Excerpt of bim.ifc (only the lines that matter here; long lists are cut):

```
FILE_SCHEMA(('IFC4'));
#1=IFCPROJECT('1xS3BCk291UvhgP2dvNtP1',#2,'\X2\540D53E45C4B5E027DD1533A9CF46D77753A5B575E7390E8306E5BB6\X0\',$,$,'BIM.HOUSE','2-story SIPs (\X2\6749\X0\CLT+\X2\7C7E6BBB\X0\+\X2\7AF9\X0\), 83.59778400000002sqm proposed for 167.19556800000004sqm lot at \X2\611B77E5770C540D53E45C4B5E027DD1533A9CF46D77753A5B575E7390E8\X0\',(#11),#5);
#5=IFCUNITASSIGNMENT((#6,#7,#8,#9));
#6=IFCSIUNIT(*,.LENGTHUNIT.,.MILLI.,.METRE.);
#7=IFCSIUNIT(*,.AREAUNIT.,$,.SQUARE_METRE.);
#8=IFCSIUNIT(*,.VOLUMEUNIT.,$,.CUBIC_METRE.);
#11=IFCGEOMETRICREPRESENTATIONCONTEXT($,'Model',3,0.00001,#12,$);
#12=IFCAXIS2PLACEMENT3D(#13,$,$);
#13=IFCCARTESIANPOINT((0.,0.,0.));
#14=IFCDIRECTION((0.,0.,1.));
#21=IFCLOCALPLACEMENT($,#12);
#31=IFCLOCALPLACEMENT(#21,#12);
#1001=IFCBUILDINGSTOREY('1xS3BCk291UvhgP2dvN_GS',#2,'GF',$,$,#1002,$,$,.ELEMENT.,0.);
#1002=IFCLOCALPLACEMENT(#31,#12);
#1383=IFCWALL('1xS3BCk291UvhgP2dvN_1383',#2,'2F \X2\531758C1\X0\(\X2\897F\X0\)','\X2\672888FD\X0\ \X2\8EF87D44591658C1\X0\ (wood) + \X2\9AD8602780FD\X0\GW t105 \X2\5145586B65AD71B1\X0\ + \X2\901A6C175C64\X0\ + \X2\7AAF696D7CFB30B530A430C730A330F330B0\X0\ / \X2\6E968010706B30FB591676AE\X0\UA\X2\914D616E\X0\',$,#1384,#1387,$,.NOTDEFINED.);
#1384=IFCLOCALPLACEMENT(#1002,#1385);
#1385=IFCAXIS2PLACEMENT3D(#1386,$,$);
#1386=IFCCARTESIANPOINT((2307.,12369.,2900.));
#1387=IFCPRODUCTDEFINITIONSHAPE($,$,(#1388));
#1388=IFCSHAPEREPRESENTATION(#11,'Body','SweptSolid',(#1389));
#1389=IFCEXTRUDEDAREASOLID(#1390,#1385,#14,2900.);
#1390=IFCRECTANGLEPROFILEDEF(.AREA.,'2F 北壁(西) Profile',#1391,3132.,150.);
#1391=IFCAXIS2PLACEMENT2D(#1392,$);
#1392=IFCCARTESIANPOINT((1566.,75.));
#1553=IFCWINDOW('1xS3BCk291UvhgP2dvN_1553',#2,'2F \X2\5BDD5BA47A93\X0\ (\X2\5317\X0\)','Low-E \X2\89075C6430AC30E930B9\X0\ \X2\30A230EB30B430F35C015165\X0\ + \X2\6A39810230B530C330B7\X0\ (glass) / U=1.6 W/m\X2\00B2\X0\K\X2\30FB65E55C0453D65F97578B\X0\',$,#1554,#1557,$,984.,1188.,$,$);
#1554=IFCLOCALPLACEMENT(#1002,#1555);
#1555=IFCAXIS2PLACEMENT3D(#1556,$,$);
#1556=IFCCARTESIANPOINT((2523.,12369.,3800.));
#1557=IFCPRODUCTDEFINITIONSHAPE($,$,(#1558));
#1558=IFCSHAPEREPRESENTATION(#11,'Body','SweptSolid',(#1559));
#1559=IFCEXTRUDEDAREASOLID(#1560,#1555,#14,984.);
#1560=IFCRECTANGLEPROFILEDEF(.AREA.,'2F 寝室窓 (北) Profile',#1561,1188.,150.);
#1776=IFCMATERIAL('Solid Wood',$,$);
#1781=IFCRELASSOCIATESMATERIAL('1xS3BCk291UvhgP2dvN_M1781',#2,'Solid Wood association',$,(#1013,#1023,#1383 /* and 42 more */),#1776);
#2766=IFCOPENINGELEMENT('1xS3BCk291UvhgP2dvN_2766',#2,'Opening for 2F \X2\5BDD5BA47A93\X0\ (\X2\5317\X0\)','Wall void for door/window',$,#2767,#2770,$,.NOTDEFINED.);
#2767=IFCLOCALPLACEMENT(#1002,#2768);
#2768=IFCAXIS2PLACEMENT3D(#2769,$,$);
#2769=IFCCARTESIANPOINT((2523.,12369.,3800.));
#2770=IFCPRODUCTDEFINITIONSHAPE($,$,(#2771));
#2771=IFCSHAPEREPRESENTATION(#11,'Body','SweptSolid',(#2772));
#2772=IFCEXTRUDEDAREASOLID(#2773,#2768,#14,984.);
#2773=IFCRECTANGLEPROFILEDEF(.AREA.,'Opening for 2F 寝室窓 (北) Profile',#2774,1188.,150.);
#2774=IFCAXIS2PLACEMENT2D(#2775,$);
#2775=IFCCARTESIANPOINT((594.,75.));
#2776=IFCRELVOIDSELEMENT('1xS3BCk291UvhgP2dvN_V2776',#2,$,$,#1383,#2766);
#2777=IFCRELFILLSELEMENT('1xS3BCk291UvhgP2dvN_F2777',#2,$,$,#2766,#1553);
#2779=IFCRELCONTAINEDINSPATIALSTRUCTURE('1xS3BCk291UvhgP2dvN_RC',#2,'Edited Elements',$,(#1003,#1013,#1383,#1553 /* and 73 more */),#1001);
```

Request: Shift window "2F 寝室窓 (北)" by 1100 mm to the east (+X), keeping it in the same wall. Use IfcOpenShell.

```python
import ifcopenshell
import ifcopenshell.api.geometry
import ifcopenshell.util.placement

model = ifcopenshell.open("bim.ifc")

window = model.by_id(1553)
opening = window.FillsVoids[0].RelatingOpeningElement
wall = opening.VoidsElements[0].RelatingBuildingElement

wall_matrix = ifcopenshell.util.placement.get_local_placement(wall.ObjectPlacement)
shift = wall_matrix[:3, 0] * 1100.0
before = ifcopenshell.util.placement.get_local_placement(window.ObjectPlacement)[:3, 3].copy()

# The window is not placed relative to its opening, so move both.
for product in (opening, window):
    matrix = ifcopenshell.util.placement.get_local_placement(product.ObjectPlacement)
    matrix[:3, 3] += shift
    ifcopenshell.api.geometry.edit_object_placement(model, product=product, matrix=matrix, is_si=False)

after = ifcopenshell.util.placement.get_local_placement(window.ObjectPlacement)[:3, 3]
print("window moved by", (after - before).round(3) + 0.0)

model.write("bim_v2.ifc")
```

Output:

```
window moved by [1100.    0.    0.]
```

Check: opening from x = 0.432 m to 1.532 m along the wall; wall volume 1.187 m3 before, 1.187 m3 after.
